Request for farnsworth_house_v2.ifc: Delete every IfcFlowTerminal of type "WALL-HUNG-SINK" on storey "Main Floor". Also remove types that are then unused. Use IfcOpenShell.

First a look at what the model holds.

```python
import ifcopenshell
import ifcopenshell.util.element

model = ifcopenshell.open("farnsworth_house_v2.ifc")
print(model.schema)
storey = next(s for s in model.by_type("IfcBuildingStorey") if s.Name == "Main Floor")
terminals = [e for e in ifcopenshell.util.element.get_decomposition(storey) if e.is_a("IfcFlowTerminal")]
seen = {}
for e in terminals:
    element_type = ifcopenshell.util.element.get_type(e)
    name = element_type.Name if element_type not in (None, e) else None
    seen[name] = seen.get(name, 0) + 1
for name, count in sorted(seen.items(), key=str):
    print(count, "x", name)
```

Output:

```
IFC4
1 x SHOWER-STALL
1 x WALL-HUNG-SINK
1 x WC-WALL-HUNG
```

```python
import ifcopenshell
import ifcopenshell.api.root
import ifcopenshell.util.element

model = ifcopenshell.open("farnsworth_house_v2.ifc")

storey = next(s for s in model.by_type("IfcBuildingStorey") if s.Name == "Main Floor")
terminals = [e for e in ifcopenshell.util.element.get_decomposition(storey) if e.is_a("IfcFlowTerminal")]
targets = [e for e in terminals if (t := ifcopenshell.util.element.get_type(e)) not in (None, e) and t.Name == "WALL-HUNG-SINK"]
types = {ifcopenshell.util.element.get_type(e) for e in targets} - {None, *targets}

for e in targets:
    ifcopenshell.api.root.remove_product(model, product=e)
print(len(targets), "removed")

unused = [t for t in types if not ifcopenshell.util.element.get_types(t)]
for t in unused:
    ifcopenshell.api.root.remove_product(model, product=t)
print(len(unused), "unused types removed")

model.write("farnsworth_house_v2-out.ifc")
```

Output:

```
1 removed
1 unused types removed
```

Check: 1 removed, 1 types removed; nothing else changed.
